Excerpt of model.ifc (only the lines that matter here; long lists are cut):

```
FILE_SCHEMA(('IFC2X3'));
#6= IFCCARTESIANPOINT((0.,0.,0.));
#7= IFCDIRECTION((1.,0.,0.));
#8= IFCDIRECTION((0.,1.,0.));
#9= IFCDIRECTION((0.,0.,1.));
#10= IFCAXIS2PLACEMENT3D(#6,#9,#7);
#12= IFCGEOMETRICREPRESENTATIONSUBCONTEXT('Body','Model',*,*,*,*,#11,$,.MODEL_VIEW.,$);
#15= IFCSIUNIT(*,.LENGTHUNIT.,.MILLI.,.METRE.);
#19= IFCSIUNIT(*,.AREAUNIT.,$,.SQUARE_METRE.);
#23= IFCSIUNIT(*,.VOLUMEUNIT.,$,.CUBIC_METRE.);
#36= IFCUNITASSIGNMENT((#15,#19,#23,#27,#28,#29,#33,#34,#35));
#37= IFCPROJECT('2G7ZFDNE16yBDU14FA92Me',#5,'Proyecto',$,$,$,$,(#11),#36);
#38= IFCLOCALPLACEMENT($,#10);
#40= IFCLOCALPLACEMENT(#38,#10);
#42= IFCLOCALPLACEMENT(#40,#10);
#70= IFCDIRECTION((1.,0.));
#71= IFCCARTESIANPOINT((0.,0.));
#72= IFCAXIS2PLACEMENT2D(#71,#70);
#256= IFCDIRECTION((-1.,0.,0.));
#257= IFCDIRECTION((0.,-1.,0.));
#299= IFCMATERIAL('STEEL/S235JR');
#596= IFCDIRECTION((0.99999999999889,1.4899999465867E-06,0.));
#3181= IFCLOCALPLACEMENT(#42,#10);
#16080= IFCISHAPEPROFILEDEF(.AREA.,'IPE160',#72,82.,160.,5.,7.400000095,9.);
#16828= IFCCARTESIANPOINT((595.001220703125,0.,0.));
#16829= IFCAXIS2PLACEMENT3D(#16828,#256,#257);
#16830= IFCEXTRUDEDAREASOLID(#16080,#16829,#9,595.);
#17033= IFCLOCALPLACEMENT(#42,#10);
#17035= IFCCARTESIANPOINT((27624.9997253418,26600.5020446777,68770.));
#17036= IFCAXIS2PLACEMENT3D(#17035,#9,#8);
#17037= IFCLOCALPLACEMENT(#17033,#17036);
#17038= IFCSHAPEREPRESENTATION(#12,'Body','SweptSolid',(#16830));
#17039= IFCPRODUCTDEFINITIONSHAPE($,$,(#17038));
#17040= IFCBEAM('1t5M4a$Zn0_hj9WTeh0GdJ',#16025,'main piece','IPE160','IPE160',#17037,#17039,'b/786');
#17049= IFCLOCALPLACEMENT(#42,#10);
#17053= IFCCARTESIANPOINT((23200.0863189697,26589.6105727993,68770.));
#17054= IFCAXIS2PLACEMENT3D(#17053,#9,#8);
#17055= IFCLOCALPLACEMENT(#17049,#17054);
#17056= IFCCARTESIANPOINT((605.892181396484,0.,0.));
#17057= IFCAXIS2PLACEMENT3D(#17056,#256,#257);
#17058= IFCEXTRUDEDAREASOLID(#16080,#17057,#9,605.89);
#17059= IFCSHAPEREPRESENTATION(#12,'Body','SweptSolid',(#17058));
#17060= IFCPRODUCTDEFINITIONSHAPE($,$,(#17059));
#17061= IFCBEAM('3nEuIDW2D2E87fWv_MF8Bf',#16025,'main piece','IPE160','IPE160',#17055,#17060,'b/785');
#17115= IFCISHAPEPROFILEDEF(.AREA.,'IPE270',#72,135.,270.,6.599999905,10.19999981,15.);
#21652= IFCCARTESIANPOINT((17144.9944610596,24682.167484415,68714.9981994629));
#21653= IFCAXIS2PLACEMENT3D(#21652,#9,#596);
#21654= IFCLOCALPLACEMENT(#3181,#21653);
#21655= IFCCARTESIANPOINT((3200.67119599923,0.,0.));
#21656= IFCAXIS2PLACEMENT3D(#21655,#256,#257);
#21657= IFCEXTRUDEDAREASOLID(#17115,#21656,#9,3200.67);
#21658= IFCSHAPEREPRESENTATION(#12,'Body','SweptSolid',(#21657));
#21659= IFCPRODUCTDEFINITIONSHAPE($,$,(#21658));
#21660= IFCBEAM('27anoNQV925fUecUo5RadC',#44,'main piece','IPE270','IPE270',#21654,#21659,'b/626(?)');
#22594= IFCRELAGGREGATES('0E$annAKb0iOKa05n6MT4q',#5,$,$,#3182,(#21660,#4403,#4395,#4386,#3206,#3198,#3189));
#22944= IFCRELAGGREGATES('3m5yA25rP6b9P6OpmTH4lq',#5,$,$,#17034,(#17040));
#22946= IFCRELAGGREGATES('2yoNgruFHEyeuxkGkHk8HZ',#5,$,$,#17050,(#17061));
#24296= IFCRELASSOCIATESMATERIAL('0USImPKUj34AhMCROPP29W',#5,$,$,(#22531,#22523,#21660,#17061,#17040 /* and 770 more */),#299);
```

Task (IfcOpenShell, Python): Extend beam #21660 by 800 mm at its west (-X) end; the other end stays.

```python
import ifcopenshell
import ifcopenshell.util.representation
import ifcopenshell.util.unit

model = ifcopenshell.open("model.ifc")
unit_scale = ifcopenshell.util.unit.calculate_unit_scale(model)

member = model.by_id(21660)
change = 0.8 / unit_scale

# The extrusion runs towards the end named, so only its depth changes.
body = ifcopenshell.util.representation.get_representation(member, "Model", "Body")
solid = body.Items[0]
old_length = solid.Depth
solid.Depth += change

print(f"length {old_length:g} -> {solid.Depth:g}")

model.write("model-out.ifc")
```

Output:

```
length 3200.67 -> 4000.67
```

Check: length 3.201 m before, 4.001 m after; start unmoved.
